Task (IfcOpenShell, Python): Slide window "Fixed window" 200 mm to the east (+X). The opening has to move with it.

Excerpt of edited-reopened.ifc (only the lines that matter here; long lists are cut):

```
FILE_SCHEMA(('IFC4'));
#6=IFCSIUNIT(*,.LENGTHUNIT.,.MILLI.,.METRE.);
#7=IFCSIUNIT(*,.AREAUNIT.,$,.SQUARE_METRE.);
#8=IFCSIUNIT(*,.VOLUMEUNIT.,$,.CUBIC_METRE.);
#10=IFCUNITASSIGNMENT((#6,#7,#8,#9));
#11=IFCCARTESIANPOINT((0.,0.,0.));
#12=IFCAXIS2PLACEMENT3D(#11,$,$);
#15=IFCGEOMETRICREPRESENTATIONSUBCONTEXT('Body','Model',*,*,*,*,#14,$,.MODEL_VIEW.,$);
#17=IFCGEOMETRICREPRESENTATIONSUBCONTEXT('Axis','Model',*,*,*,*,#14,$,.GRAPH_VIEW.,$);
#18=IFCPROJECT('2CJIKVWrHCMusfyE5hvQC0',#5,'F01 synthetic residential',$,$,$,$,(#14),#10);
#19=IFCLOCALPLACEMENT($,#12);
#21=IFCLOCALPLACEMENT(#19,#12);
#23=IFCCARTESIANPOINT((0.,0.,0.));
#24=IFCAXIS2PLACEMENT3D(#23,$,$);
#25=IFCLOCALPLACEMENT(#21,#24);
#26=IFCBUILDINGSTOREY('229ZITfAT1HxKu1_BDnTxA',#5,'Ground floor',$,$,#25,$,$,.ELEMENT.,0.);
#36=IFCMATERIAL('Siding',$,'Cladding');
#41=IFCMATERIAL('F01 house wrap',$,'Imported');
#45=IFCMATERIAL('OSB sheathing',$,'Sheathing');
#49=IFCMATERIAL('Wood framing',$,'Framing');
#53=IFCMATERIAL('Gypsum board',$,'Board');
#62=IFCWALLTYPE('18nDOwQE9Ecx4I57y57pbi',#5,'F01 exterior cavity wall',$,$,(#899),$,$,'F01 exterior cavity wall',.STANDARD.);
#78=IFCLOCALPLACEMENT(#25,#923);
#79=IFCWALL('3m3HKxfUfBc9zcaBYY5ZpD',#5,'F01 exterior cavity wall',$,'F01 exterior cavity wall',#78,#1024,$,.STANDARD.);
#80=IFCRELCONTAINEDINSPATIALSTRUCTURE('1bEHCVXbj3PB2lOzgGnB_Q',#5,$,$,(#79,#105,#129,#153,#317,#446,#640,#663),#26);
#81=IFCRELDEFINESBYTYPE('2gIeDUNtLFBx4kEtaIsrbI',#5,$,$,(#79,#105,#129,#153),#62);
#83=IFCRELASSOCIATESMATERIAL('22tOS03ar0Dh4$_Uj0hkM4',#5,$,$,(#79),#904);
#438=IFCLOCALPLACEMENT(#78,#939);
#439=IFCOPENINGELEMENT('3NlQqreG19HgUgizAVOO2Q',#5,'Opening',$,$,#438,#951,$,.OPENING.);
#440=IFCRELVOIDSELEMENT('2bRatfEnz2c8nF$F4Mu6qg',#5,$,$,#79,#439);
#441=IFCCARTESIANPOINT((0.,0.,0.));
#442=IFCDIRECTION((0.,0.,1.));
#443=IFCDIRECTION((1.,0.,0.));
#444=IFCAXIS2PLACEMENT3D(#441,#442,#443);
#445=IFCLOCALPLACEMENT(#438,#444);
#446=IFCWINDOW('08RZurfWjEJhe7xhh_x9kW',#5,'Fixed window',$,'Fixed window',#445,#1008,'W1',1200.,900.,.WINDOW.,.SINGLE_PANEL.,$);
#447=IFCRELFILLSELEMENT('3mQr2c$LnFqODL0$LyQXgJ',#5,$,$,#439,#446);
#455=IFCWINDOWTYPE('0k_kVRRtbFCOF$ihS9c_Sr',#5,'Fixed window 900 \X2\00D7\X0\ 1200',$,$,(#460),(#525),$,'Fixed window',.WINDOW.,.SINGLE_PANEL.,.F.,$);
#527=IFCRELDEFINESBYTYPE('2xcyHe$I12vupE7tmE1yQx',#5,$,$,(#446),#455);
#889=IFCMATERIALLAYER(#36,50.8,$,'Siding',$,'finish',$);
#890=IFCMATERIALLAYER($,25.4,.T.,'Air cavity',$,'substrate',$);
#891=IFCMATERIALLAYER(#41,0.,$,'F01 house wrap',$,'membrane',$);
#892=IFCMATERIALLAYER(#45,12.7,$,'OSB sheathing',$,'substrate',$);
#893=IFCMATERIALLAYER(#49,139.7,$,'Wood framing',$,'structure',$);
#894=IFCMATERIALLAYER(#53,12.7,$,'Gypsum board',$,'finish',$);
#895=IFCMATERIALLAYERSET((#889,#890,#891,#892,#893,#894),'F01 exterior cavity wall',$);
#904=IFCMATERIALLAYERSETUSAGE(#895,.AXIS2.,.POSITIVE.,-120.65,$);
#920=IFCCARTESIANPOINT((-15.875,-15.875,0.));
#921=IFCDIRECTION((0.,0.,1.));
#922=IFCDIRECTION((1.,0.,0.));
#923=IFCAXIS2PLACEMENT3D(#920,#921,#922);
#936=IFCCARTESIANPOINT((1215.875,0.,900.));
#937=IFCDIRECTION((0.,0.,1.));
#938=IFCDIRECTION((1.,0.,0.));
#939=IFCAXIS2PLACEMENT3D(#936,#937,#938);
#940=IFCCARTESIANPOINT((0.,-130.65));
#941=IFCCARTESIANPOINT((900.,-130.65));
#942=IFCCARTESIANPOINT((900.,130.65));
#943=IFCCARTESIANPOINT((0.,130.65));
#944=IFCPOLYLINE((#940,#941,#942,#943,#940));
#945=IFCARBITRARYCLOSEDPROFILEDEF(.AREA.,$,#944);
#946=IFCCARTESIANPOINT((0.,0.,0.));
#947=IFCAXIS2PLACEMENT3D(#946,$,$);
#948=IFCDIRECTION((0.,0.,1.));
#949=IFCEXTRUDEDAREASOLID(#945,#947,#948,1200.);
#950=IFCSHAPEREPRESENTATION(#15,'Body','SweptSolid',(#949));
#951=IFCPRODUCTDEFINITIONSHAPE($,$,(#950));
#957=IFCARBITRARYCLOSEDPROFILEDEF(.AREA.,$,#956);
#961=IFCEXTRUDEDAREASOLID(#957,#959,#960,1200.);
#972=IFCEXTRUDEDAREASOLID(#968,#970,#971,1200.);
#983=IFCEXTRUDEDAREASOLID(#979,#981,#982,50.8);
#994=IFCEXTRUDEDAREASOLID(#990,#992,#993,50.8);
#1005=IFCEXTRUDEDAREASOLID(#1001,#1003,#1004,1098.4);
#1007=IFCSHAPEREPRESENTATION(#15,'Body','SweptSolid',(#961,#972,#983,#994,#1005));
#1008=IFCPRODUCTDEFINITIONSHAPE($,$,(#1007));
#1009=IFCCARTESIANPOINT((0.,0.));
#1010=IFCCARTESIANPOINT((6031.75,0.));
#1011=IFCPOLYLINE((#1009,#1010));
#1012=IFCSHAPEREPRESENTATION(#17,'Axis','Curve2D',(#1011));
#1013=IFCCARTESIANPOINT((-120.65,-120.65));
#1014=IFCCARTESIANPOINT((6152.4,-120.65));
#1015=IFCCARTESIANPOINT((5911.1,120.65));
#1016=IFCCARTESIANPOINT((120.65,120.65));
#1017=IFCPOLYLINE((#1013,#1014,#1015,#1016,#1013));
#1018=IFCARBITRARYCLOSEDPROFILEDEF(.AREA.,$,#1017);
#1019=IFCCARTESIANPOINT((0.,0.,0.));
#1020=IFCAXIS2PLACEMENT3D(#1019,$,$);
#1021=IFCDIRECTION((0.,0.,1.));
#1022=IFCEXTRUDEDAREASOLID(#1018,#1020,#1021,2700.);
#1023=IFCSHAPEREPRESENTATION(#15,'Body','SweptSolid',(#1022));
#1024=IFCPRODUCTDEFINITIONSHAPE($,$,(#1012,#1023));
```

```python
import ifcopenshell
import ifcopenshell.api.geometry
import ifcopenshell.util.placement
import ifcopenshell.util.unit

model = ifcopenshell.open("edited-reopened.ifc")
unit_scale = ifcopenshell.util.unit.calculate_unit_scale(model)

window = model.by_guid("08RZurfWjEJhe7xhh_x9kW")
opening = window.FillsVoids[0].RelatingOpeningElement
wall = opening.VoidsElements[0].RelatingBuildingElement

wall_matrix = ifcopenshell.util.placement.get_local_placement(wall.ObjectPlacement)
shift = wall_matrix[:3, 0] * 0.2 / unit_scale
before = ifcopenshell.util.placement.get_local_placement(window.ObjectPlacement)[:3, 3].copy()

# The window is placed relative to its opening, so it follows when the opening moves.
matrix = ifcopenshell.util.placement.get_local_placement(opening.ObjectPlacement)
matrix[:3, 3] += shift
ifcopenshell.api.geometry.edit_object_placement(
    model, product=opening, matrix=matrix, is_si=False, should_transform_children=True
)

after = ifcopenshell.util.placement.get_local_placement(window.ObjectPlacement)[:3, 3]
print("window moved by", (after - before).round(3) + 0.0)

model.write("edited-reopened-out.ifc")
```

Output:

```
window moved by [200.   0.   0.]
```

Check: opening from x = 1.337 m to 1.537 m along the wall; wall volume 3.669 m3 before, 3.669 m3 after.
